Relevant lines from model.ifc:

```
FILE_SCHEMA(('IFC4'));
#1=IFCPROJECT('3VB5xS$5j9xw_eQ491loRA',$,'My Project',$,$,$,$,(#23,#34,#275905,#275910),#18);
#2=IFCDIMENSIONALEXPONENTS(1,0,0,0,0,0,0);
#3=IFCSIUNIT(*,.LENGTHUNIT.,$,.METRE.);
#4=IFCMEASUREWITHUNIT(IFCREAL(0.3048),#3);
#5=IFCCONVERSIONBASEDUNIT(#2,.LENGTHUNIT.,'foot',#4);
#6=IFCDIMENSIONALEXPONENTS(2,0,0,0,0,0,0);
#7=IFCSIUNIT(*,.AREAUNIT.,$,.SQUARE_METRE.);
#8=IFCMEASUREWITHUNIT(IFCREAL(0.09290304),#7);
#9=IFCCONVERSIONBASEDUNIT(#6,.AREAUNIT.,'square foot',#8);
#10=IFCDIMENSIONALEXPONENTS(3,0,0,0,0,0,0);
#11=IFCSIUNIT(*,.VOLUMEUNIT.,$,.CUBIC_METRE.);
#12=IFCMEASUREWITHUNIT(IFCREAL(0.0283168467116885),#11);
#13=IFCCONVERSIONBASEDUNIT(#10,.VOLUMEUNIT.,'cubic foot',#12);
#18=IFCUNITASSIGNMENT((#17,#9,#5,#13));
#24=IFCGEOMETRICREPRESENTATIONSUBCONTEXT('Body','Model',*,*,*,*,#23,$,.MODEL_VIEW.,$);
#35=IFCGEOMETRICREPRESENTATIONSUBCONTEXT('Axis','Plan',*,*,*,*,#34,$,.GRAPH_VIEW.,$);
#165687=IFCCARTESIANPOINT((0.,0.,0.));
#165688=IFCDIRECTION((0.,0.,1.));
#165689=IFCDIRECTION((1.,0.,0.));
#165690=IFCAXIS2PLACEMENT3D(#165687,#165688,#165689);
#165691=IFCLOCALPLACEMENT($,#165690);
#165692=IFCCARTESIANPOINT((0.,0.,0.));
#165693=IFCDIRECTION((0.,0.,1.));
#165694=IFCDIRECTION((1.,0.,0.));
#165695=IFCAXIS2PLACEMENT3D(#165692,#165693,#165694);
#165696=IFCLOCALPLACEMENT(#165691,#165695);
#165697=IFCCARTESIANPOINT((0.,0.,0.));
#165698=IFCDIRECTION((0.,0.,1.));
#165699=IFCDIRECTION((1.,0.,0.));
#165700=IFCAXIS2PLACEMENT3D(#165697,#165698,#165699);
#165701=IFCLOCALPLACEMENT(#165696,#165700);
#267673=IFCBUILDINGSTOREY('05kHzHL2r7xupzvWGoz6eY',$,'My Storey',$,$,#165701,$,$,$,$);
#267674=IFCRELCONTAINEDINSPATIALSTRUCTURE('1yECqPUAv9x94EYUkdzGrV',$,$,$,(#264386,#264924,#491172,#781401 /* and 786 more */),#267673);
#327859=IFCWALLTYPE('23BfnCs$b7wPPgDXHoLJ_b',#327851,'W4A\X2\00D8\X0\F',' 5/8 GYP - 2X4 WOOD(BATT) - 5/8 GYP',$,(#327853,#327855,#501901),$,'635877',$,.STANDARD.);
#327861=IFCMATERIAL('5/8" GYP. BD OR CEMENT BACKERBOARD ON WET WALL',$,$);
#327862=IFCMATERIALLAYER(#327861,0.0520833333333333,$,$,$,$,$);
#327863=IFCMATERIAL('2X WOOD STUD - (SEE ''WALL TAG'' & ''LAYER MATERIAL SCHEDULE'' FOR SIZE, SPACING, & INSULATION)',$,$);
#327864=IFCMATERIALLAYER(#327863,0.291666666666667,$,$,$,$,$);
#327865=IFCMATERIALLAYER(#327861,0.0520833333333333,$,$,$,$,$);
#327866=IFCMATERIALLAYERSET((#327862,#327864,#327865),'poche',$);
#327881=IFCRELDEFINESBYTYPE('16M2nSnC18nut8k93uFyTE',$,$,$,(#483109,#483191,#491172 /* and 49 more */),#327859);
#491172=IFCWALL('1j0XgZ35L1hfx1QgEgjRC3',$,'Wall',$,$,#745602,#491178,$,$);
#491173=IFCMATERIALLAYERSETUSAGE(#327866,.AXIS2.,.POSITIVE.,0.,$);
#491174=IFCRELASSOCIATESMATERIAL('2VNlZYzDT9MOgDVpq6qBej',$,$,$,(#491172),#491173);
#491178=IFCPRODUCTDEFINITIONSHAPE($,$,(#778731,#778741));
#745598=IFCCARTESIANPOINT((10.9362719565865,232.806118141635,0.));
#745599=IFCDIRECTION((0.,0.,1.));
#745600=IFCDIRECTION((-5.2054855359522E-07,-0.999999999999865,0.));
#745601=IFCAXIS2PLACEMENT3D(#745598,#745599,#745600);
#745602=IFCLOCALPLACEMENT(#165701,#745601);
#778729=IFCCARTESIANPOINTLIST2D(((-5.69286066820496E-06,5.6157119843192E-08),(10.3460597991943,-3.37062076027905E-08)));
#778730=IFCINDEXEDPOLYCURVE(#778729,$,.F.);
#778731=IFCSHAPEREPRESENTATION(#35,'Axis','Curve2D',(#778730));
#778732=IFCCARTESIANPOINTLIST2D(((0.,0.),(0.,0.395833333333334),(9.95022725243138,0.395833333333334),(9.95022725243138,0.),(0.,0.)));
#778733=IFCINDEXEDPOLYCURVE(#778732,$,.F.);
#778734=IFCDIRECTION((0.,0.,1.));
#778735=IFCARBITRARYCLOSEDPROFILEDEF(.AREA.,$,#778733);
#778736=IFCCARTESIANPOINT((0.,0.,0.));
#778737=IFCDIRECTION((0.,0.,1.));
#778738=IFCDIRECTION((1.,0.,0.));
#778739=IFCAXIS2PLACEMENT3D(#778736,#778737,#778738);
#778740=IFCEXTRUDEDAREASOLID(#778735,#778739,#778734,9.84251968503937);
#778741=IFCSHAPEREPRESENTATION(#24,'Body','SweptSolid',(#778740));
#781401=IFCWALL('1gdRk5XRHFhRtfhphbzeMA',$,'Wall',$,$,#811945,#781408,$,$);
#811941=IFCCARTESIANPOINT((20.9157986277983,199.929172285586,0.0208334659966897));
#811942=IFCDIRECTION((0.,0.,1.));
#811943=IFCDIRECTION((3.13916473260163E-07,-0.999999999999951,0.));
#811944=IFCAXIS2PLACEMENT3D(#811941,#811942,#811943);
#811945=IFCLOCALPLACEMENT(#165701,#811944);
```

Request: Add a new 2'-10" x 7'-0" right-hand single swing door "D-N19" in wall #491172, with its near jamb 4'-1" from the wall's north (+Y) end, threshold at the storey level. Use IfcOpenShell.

```python
import numpy as np
import ifcopenshell
import ifcopenshell.api.feature
import ifcopenshell.api.geometry
import ifcopenshell.api.root
import ifcopenshell.api.spatial
import ifcopenshell.geom
import ifcopenshell.util.element
import ifcopenshell.util.placement
import ifcopenshell.util.representation
import ifcopenshell.util.shape
import ifcopenshell.util.unit

model = ifcopenshell.open("model.ifc")
unit_scale = ifcopenshell.util.unit.calculate_unit_scale(model)
settings = ifcopenshell.geom.settings()


def volume(element):
    """Net volume in cubic metres, openings subtracted."""
    shape = ifcopenshell.geom.create_shape(settings, element)
    return ifcopenshell.util.shape.get_volume(shape.geometry)


wall = model.by_guid("1j0XgZ35L1hfx1QgEgjRC3")
storey = ifcopenshell.util.element.get_container(wall, ifc_class="IfcBuildingStorey")
context = ifcopenshell.util.representation.get_context(model, "Model", "Body", "MODEL_VIEW")
before = volume(wall)

width, height, from_end, sill = 0.8636, 2.1336, 1.2446, 0.0  # metres

# The wall runs along its own X axis, and the end named is its -X end.
wall_shape = ifcopenshell.geom.create_shape(settings, wall)
x, y, z = ifcopenshell.util.shape.get_vertices(wall_shape.geometry).T
start = x.min() + from_end
face, thickness = float(y.min()), float(y.max() - y.min())
wall_matrix = ifcopenshell.util.placement.get_local_placement(wall.ObjectPlacement)
level = ifcopenshell.util.placement.get_local_placement(storey.ObjectPlacement)[2, 3]


def in_wall(x, y):
    """Placement at x, y metres in the wall's axes, at sill height."""
    matrix = wall_matrix.copy()
    matrix[:, 3] = wall_matrix @ np.array([x / unit_scale, y / unit_scale, 0.0, 1.0])
    matrix[2, 3] = level + sill / unit_scale
    return matrix


# Opening: a box that overshoots both wall faces by 50 mm.
opening = ifcopenshell.api.root.create_entity(model, ifc_class="IfcOpeningElement", predefined_type="OPENING")
box = ifcopenshell.api.geometry.add_wall_representation(
    model, context=context, length=width, height=height, thickness=thickness + 0.1
)
ifcopenshell.api.geometry.assign_representation(model, product=opening, representation=box)
ifcopenshell.api.geometry.edit_object_placement(model, product=opening, matrix=in_wall(start, face - 0.05), is_si=False)
ifcopenshell.api.feature.add_feature(model, feature=opening, element=wall)

door = ifcopenshell.api.root.create_entity(model, ifc_class="IfcDoor", name="D-N19", predefined_type="DOOR")
door.OverallWidth, door.OverallHeight = width / unit_scale, height / unit_scale
door.OperationType = "SINGLE_SWING_RIGHT"
body = ifcopenshell.api.geometry.add_door_representation(
    model,
    context=context,
    overall_width=door.OverallWidth,
    overall_height=door.OverallHeight,
    operation_type="SINGLE_SWING_RIGHT",
    lining_properties={"LiningDepth": thickness / unit_scale, "ThresholdDepth": thickness / unit_scale},
)
ifcopenshell.api.geometry.assign_representation(model, product=door, representation=body)
ifcopenshell.api.spatial.assign_container(model, products=[door], relating_structure=storey)
ifcopenshell.api.feature.add_filling(model, opening=opening, element=door)

# The lining spans the wall, so the door starts at the wall face.
ifcopenshell.api.geometry.edit_object_placement(model, product=door, matrix=in_wall(start, face), is_si=False)

after = volume(wall)

print(f"wall volume {before:.3f} -> {after:.3f} m3")

model.write("model_edited.ifc")
```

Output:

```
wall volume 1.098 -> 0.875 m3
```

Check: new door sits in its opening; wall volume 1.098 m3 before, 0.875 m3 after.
